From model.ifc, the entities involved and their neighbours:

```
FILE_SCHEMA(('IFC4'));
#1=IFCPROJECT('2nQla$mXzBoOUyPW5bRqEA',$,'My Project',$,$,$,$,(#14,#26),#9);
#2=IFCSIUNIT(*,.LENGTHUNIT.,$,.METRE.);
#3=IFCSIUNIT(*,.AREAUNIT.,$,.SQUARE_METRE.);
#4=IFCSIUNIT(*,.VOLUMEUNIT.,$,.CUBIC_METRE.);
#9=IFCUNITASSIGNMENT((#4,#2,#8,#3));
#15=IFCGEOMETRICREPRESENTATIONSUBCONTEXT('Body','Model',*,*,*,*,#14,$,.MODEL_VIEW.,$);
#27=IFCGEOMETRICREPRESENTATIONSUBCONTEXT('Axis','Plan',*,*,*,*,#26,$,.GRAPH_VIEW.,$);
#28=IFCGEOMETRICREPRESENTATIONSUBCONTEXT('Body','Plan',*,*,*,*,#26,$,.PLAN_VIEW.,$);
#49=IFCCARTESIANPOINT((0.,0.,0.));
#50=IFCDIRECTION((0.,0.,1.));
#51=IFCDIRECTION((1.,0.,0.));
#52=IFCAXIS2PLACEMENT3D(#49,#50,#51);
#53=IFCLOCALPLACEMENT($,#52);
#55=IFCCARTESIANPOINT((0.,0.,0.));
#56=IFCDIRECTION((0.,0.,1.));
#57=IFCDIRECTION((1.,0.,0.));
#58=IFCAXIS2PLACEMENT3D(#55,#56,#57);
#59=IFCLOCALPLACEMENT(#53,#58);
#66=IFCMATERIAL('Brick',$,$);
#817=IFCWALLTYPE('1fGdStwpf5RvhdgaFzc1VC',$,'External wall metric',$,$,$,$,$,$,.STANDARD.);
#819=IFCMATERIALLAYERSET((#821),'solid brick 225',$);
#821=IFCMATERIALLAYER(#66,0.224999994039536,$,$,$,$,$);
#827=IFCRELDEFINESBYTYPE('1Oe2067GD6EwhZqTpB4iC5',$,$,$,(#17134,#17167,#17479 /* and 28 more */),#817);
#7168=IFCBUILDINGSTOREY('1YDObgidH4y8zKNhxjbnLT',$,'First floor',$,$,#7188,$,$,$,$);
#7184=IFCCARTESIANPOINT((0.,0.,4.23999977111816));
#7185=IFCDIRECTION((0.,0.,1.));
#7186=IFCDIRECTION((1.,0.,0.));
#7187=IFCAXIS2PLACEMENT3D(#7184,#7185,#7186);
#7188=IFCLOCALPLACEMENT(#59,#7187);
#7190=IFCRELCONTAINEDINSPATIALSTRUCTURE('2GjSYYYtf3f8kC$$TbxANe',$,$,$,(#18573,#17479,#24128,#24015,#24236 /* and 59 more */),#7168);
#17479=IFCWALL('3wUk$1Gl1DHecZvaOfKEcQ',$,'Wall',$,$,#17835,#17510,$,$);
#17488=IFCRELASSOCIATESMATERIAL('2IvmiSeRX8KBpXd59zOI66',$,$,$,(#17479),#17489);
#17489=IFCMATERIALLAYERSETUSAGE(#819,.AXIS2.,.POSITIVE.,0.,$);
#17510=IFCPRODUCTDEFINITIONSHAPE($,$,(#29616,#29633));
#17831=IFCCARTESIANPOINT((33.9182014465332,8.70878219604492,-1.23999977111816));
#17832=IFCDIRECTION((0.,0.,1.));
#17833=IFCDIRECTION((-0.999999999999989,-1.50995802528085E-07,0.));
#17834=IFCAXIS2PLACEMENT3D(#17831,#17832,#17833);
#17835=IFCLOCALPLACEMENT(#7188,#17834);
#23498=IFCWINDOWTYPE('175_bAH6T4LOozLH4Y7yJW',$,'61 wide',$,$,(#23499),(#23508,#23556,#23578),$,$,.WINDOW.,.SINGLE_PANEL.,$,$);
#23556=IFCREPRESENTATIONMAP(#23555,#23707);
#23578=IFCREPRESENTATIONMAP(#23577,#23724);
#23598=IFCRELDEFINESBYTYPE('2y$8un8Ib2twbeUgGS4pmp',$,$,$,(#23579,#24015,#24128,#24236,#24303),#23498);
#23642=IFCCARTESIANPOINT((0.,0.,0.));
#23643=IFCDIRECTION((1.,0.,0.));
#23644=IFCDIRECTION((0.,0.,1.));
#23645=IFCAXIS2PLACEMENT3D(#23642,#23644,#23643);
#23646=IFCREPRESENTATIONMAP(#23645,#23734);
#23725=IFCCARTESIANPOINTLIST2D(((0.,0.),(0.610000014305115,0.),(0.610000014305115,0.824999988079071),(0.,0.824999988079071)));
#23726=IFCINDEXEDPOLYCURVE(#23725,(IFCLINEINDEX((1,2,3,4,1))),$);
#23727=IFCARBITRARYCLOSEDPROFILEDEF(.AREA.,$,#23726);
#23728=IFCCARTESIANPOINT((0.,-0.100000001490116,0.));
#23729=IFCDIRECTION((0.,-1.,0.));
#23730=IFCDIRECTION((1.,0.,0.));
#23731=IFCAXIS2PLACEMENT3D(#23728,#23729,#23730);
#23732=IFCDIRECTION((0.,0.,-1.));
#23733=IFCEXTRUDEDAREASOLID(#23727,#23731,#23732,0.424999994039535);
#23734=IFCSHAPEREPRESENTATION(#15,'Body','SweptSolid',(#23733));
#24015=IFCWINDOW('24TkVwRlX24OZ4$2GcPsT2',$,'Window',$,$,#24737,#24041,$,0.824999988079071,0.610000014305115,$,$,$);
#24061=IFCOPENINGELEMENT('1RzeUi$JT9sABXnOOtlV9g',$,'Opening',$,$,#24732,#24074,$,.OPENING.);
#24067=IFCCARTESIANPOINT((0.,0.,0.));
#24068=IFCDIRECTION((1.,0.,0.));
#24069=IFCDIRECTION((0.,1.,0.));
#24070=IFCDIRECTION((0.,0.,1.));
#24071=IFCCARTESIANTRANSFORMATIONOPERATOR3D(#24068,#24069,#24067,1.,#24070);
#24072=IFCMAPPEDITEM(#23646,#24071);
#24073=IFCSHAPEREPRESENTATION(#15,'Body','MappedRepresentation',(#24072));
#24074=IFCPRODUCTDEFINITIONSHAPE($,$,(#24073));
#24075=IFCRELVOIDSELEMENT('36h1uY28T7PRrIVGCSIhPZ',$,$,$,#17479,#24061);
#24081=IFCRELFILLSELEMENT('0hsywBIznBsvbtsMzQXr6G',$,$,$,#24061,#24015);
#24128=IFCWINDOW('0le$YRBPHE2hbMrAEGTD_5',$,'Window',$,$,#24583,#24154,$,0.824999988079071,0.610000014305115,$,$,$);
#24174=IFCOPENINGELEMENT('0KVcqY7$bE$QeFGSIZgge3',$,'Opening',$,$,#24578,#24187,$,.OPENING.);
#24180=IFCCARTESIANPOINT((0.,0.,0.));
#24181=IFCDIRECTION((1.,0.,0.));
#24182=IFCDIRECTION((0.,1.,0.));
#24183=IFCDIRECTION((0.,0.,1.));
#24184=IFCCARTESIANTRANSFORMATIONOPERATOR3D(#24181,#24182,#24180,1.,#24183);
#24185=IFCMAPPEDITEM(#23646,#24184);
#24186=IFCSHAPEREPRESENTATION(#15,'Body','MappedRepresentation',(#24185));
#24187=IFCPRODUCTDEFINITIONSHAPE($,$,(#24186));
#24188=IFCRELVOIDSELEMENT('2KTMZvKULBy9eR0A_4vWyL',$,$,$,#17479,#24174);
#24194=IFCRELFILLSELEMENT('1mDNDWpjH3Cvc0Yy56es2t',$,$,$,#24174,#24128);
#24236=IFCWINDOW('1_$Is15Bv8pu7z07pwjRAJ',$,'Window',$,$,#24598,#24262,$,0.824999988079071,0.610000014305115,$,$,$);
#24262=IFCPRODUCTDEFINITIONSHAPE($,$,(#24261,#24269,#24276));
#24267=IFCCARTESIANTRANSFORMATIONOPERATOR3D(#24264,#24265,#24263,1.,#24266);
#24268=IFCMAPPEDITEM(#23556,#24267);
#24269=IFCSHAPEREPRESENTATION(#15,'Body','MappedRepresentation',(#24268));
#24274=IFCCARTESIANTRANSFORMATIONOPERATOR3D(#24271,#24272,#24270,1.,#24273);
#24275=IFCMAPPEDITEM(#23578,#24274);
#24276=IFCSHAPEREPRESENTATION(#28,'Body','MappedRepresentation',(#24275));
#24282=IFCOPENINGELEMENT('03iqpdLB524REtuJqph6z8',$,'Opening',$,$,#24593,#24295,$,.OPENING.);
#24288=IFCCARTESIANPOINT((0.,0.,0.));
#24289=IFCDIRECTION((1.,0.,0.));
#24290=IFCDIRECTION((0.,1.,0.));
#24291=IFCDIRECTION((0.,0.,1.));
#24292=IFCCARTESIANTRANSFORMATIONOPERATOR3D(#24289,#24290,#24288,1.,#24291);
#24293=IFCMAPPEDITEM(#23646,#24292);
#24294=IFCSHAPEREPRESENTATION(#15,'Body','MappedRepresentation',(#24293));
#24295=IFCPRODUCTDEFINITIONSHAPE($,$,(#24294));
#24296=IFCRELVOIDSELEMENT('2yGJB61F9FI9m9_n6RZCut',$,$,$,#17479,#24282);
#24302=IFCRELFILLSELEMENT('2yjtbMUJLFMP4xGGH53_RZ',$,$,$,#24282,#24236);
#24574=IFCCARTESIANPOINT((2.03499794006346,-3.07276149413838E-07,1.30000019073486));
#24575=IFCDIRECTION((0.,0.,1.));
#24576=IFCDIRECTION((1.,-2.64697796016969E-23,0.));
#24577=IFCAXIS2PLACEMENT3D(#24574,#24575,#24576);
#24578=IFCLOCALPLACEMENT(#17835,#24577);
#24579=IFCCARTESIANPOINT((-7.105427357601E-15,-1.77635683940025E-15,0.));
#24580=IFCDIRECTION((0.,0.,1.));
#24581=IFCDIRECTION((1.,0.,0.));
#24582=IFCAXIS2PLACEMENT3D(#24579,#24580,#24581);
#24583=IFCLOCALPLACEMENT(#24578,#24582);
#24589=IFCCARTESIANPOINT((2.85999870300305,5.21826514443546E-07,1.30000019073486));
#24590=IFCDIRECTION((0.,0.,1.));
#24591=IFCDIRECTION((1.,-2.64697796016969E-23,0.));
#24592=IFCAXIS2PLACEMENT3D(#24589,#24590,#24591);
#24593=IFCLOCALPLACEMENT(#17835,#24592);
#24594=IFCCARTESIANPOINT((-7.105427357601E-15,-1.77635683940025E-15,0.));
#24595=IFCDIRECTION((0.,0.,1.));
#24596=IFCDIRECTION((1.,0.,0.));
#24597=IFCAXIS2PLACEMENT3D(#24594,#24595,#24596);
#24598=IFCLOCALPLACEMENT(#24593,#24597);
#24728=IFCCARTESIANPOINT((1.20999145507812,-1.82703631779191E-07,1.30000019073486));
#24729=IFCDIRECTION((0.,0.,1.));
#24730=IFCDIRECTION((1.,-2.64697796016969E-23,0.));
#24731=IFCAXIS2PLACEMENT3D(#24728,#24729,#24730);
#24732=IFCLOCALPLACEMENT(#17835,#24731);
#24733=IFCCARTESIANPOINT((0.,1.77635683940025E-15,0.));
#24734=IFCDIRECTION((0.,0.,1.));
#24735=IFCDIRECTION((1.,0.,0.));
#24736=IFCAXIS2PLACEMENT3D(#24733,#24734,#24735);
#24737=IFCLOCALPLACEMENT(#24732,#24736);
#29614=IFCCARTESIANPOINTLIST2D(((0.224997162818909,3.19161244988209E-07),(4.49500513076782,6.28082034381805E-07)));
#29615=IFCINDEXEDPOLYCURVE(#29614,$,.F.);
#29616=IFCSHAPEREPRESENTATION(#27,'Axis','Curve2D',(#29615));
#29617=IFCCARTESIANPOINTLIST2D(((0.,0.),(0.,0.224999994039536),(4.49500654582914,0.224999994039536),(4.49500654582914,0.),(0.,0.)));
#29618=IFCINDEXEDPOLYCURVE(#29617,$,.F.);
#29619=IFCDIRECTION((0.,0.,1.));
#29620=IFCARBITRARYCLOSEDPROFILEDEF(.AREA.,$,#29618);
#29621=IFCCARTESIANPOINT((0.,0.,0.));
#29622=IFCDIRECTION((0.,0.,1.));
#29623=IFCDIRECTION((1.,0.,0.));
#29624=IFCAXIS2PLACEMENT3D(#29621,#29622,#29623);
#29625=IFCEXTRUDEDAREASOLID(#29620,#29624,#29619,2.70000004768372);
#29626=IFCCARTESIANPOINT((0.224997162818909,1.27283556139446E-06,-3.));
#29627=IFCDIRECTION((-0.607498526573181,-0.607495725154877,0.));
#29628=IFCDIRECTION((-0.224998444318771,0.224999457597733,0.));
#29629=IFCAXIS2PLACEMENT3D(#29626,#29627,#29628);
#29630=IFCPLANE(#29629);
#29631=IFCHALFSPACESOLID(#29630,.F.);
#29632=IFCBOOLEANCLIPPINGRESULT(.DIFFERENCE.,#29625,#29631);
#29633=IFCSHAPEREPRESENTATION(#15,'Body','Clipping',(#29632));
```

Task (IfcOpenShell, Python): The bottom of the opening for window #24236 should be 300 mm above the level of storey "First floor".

```python
import numpy as np
import ifcopenshell
import ifcopenshell.api.geometry
import ifcopenshell.geom
import ifcopenshell.util.element
import ifcopenshell.util.placement
import ifcopenshell.util.shape
import ifcopenshell.util.unit

model = ifcopenshell.open("model.ifc")
unit_scale = ifcopenshell.util.unit.calculate_unit_scale(model)

window = model.by_id(24236)
opening = window.FillsVoids[0].RelatingOpeningElement
storey = ifcopenshell.util.element.get_container(window, ifc_class="IfcBuildingStorey")
level = ifcopenshell.util.placement.get_local_placement(storey.ObjectPlacement)[2, 3]

# The opening's origin need not be at the sill, so measure its lowest point.
shape = ifcopenshell.geom.create_shape(ifcopenshell.geom.settings(), opening)
bottom = ifcopenshell.util.shape.get_shape_bottom_elevation(shape, shape.geometry) / unit_scale
dz = level + 0.3 / unit_scale - bottom

shift = np.array([0.0, 0.0, dz])
# The window is placed relative to its opening, so it follows when the opening moves.
matrix = ifcopenshell.util.placement.get_local_placement(opening.ObjectPlacement)
matrix[:3, 3] += shift
ifcopenshell.api.geometry.edit_object_placement(
    model, product=opening, matrix=matrix, is_si=False, should_transform_children=True
)

print(f"moved by {dz * unit_scale:+.3f} m")

model.write("model_v2.ifc")
```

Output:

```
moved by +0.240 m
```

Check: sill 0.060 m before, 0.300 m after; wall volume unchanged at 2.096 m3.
